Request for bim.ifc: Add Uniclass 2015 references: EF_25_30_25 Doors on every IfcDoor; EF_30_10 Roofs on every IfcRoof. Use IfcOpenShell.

First a look at what the model holds.

```python
import ifcopenshell

model = ifcopenshell.open("bim.ifc")
print(model.schema)
print("classifications:", [c.Name for c in model.by_type("IfcClassification")])
for ifc_class in ("IfcDoor", "IfcRoof", "IfcStair", "IfcWall", "IfcWindow"):
    print(ifc_class, len(model.by_type(ifc_class)))
```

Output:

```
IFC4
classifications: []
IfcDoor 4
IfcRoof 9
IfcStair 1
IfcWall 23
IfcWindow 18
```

```python
import ifcopenshell
import ifcopenshell.api.classification

model = ifcopenshell.open("bim.ifc")

system = ifcopenshell.api.classification.add_classification(model, classification="Uniclass 2015")

codes = {
    "IfcDoor": ("EF_25_30_25", "Doors"),
    "IfcRoof": ("EF_30_10", "Roofs"),
}
for ifc_class, (code, name) in codes.items():
    products = model.by_type(ifc_class)
    ifcopenshell.api.classification.add_reference(
        model, products=products, classification=system, identification=code, name=name
    )
    print(code, len(products))

model.write("bim_v2.ifc")
```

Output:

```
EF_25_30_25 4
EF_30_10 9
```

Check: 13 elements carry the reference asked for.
